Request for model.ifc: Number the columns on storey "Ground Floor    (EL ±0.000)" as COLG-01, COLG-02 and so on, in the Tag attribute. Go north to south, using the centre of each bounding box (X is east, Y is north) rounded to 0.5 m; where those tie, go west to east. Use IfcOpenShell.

First a look at what the model holds.

```python
import ifcopenshell
import ifcopenshell.util.element
import ifcopenshell.util.placement

model = ifcopenshell.open("model.ifc")
print(model.schema)
storey = next(s for s in model.by_type("IfcBuildingStorey") if s.Name == "Ground Floor    (EL ±0.000)")
columns = [e for e in ifcopenshell.util.element.get_decomposition(storey) if e.is_a("IfcColumn")]
for e in sorted(columns, key=lambda e: e.id()):
    origin = ifcopenshell.util.placement.get_local_placement(e.ObjectPlacement)[:3, 3]
    print(e.id(), e.Tag, e.Name, origin.round(2) + 0.0, sep=" | ")
```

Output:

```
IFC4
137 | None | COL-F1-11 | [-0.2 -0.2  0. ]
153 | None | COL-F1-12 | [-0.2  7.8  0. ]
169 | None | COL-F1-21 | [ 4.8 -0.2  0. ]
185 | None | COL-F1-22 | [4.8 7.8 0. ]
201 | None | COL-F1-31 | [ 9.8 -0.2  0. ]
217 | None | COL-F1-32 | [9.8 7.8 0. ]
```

```python
import ifcopenshell
import ifcopenshell.geom
import ifcopenshell.util.element
import ifcopenshell.util.shape

model = ifcopenshell.open("model.ifc")
settings = ifcopenshell.geom.settings()
settings.set("use-world-coords", True)


def centre(element):
    shape = ifcopenshell.geom.create_shape(settings, element)
    return ifcopenshell.util.shape.get_bbox_centroid(shape.geometry)


storey = next(s for s in model.by_type("IfcBuildingStorey") if s.Name == "Ground Floor    (EL ±0.000)")
columns = [e for e in ifcopenshell.util.element.get_decomposition(storey) if e.is_a("IfcColumn")]

# Insertion points can sit at a corner or the storey origin, so sort by the geometry (in metres).
centres = {e: centre(e) for e in columns}
columns.sort(key=lambda e: (-round(centres[e][1] / 0.5), centres[e][0]))

for i, e in enumerate(columns, start=1):
    number = f"COLG-{i:02d}"
    e.Tag = number
    print(e.id(), number)

model.write("model_updated.ifc")
```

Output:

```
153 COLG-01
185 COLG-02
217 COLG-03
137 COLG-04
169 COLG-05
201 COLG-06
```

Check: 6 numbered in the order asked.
